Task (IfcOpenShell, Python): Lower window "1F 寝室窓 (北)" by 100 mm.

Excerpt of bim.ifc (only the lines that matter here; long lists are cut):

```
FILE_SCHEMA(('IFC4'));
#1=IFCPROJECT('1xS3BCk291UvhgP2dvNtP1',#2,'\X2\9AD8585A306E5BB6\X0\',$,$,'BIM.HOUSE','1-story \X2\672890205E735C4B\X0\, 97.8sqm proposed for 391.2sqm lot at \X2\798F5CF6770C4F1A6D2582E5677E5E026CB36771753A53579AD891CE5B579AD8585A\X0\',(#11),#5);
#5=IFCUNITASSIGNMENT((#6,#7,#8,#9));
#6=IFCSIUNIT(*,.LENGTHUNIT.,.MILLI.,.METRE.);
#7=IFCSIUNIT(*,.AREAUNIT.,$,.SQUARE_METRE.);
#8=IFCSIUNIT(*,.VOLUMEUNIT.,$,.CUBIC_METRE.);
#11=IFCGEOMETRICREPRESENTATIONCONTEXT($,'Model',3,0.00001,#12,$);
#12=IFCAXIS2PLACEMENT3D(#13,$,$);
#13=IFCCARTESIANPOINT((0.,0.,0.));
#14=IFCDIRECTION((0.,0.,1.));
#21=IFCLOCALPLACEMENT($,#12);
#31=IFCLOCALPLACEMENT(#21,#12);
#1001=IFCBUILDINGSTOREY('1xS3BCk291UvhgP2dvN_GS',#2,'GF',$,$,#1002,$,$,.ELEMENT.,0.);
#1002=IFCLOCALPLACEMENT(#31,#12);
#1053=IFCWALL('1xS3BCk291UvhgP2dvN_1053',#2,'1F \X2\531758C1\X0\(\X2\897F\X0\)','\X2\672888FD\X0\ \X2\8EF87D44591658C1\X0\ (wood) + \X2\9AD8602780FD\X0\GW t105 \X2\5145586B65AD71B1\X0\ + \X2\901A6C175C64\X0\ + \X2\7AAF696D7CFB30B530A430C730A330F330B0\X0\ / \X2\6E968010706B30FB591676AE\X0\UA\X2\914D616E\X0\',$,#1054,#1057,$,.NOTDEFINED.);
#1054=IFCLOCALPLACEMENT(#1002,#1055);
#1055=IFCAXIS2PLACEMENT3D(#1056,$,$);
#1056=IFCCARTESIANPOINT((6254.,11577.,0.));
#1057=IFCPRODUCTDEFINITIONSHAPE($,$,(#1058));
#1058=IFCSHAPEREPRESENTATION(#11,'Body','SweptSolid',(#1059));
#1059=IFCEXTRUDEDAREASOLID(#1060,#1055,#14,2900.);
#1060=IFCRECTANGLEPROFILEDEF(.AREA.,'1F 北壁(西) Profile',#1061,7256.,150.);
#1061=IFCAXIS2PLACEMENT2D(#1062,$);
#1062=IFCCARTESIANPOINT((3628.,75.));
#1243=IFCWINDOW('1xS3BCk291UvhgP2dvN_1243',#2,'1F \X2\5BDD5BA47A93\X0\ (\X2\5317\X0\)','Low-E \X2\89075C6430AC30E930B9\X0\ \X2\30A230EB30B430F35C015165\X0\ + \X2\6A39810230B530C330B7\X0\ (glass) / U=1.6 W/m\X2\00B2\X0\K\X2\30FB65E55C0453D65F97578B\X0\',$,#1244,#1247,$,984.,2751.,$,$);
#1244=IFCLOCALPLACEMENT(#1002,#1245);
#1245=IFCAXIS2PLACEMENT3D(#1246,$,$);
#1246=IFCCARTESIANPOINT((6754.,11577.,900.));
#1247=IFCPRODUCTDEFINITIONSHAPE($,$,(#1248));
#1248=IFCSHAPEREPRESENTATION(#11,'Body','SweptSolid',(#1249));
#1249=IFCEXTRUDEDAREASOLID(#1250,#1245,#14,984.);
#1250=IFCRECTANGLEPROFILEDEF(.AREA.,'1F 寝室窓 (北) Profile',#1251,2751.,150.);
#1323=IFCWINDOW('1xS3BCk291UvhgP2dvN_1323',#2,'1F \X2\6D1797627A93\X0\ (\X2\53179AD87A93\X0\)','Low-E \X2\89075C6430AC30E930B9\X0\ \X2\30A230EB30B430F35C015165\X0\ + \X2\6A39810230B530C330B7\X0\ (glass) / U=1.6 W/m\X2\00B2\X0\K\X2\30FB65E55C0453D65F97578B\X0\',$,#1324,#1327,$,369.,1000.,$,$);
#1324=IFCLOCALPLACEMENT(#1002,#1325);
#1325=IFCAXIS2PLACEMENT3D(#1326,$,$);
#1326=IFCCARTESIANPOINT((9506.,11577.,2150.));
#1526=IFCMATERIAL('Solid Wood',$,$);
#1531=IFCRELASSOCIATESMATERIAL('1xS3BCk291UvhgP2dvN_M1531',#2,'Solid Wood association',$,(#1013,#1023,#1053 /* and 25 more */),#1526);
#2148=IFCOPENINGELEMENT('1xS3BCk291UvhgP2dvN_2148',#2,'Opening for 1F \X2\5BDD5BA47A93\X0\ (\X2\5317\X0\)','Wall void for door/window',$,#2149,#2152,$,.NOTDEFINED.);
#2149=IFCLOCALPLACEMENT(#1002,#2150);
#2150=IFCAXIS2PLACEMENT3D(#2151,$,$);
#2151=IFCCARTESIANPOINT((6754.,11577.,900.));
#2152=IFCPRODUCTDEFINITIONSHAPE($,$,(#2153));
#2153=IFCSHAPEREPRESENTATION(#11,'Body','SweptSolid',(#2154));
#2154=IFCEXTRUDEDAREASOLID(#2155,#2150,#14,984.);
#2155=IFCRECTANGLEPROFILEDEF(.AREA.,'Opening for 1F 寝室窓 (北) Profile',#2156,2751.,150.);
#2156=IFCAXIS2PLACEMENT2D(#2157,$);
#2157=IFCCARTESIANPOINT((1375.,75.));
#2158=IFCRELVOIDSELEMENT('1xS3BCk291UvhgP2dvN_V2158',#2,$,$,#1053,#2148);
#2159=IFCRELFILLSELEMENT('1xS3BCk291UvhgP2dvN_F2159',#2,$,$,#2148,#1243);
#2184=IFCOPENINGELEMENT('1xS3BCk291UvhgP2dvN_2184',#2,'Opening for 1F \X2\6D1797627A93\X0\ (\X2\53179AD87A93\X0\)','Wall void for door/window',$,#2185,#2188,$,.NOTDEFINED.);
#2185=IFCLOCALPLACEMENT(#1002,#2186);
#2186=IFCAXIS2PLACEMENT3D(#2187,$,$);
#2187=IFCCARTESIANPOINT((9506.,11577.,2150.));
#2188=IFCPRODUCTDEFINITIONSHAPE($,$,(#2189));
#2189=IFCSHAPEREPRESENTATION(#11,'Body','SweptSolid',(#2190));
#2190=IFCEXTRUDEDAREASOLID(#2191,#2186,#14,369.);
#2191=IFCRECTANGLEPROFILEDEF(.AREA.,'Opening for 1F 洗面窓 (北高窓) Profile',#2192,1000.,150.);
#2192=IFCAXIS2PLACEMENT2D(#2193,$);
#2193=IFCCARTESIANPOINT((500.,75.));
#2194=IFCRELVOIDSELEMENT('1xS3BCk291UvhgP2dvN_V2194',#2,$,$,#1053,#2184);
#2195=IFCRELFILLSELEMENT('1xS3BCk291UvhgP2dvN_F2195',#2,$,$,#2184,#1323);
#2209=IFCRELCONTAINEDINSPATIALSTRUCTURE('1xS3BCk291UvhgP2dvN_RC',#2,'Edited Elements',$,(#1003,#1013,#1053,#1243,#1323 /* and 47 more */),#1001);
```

```python
import numpy as np
import ifcopenshell
import ifcopenshell.api.geometry
import ifcopenshell.util.placement
import ifcopenshell.util.unit

model = ifcopenshell.open("bim.ifc")
unit_scale = ifcopenshell.util.unit.calculate_unit_scale(model)

window = model.by_id(1243)
opening = window.FillsVoids[0].RelatingOpeningElement
dz = -0.1 / unit_scale

shift = np.array([0.0, 0.0, dz])
# The window is not placed relative to its opening, so move both.
for product in (opening, window):
    matrix = ifcopenshell.util.placement.get_local_placement(product.ObjectPlacement)
    matrix[:3, 3] += shift
    ifcopenshell.api.geometry.edit_object_placement(model, product=product, matrix=matrix, is_si=False)

print(f"moved by {dz * unit_scale:+.3f} m")

model.write("bim_v2.ifc")
```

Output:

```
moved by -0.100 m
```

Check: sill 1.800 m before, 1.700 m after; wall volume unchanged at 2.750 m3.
